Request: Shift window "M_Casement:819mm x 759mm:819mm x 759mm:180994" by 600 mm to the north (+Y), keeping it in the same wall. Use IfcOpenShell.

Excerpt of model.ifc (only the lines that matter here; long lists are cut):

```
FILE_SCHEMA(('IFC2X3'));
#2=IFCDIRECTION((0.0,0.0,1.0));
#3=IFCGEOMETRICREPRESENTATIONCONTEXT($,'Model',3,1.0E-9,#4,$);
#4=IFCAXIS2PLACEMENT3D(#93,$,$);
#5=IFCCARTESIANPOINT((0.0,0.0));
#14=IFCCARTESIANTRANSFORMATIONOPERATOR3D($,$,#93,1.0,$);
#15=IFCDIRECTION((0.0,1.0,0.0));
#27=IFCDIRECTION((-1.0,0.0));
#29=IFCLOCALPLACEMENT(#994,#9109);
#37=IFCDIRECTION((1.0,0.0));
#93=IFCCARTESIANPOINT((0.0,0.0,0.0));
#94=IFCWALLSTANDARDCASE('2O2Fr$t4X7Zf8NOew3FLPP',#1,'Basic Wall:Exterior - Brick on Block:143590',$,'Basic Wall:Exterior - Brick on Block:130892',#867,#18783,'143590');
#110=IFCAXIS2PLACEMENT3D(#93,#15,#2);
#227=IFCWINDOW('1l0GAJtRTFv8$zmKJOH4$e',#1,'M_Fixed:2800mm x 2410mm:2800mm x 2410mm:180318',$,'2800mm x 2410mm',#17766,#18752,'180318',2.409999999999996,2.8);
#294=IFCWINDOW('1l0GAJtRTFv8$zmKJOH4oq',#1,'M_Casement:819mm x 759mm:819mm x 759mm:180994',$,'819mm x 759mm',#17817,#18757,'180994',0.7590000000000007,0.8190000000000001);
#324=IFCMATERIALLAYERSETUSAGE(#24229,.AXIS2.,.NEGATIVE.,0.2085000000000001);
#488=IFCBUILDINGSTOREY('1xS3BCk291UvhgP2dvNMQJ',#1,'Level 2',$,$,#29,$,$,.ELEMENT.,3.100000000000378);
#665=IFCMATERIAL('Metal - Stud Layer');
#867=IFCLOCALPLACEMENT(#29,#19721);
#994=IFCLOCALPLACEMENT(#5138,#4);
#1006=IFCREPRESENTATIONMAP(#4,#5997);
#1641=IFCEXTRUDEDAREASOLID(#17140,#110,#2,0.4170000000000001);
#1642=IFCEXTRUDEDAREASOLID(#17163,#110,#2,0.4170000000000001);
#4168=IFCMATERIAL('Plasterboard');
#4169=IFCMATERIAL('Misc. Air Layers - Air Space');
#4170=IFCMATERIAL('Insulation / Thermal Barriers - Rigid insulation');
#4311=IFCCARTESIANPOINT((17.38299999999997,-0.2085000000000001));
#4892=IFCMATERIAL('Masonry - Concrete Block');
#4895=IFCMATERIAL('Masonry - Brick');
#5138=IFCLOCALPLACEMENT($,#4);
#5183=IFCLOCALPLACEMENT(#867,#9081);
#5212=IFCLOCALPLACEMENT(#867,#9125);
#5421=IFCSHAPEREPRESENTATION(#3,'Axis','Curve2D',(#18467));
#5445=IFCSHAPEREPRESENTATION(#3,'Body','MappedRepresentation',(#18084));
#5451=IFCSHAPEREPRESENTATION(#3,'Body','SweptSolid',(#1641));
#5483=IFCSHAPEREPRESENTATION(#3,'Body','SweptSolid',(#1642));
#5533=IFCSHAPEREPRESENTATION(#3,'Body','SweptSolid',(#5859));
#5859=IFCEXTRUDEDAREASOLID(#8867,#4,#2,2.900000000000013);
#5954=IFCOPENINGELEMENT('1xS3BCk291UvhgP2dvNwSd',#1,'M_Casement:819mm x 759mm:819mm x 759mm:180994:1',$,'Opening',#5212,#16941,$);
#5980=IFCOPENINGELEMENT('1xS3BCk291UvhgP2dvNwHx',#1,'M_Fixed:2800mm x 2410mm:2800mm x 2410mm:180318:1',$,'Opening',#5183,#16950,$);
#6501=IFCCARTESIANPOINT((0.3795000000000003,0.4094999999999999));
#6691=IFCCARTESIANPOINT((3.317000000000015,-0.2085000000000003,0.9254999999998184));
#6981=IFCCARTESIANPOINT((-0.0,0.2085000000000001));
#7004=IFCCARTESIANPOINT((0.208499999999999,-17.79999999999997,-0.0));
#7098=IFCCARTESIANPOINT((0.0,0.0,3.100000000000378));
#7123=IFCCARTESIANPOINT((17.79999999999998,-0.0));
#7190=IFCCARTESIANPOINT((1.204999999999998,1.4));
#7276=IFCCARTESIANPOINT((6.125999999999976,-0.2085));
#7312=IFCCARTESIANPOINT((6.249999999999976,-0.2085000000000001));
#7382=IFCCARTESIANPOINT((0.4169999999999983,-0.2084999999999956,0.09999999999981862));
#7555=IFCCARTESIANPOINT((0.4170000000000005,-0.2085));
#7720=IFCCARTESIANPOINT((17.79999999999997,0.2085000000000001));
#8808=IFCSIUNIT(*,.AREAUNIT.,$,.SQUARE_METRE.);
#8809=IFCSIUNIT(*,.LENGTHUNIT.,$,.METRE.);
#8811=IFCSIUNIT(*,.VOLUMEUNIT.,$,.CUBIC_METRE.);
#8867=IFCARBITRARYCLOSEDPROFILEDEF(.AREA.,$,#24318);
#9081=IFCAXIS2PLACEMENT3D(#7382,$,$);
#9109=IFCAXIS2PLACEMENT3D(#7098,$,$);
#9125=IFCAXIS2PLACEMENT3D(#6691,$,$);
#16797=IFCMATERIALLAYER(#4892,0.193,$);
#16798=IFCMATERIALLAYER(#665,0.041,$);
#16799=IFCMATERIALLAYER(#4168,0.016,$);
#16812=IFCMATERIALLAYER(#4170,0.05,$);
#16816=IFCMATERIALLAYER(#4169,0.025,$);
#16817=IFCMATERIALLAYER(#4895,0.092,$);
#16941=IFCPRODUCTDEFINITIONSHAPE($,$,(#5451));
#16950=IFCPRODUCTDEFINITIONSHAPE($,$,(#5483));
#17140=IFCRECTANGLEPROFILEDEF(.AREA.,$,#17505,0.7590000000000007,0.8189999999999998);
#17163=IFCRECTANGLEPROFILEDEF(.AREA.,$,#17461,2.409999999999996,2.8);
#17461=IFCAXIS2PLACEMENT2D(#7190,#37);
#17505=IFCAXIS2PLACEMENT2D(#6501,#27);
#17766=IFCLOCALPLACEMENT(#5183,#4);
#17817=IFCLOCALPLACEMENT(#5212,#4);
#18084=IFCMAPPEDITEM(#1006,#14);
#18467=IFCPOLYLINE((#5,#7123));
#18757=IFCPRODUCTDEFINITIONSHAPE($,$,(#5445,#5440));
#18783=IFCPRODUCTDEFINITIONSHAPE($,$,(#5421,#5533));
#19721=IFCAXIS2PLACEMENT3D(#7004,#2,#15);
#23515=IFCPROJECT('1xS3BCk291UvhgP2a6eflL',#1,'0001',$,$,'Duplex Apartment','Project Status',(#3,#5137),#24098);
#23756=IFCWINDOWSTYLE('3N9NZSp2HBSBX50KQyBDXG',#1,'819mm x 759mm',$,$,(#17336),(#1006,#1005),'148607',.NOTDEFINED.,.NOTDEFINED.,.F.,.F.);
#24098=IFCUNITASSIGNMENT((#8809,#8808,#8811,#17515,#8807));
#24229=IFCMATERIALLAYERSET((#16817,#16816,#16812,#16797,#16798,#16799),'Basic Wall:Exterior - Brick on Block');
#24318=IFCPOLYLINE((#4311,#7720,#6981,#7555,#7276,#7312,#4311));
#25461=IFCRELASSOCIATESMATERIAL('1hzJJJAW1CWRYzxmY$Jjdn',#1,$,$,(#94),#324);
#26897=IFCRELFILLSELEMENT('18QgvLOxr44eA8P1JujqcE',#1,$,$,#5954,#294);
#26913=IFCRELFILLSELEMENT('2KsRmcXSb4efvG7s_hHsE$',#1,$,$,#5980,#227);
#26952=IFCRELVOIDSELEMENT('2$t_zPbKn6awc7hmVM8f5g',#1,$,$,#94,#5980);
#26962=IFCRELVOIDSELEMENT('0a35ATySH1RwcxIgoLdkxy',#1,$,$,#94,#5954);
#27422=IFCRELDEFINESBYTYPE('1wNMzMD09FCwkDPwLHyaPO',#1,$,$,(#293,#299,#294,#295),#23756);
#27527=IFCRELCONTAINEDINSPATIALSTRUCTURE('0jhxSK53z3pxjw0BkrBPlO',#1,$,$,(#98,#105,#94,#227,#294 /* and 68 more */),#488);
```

```python
import ifcopenshell
import ifcopenshell.api.geometry
import ifcopenshell.util.placement
import ifcopenshell.util.unit

model = ifcopenshell.open("model.ifc")
unit_scale = ifcopenshell.util.unit.calculate_unit_scale(model)

window = model.by_id(294)
opening = window.FillsVoids[0].RelatingOpeningElement
wall = opening.VoidsElements[0].RelatingBuildingElement

wall_matrix = ifcopenshell.util.placement.get_local_placement(wall.ObjectPlacement)
shift = wall_matrix[:3, 0] * 0.6 / unit_scale
before = ifcopenshell.util.placement.get_local_placement(window.ObjectPlacement)[:3, 3].copy()

# The window is placed relative to its opening, so it follows when the opening moves.
matrix = ifcopenshell.util.placement.get_local_placement(opening.ObjectPlacement)
matrix[:3, 3] += shift
ifcopenshell.api.geometry.edit_object_placement(
    model, product=opening, matrix=matrix, is_si=False, should_transform_children=True
)

after = ifcopenshell.util.placement.get_local_placement(window.ObjectPlacement)[:3, 3]
print("window moved by", (after - before).round(3) + 0.0)

model.write("model_rev.ifc")
```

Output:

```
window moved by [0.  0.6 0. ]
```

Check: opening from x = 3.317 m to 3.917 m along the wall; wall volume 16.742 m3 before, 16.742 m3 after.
